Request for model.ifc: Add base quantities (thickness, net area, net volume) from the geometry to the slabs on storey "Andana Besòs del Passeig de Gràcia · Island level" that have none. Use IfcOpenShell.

First a look at what the model holds.

```python
import ifcopenshell
import ifcopenshell.util.element
import ifcopenshell.util.unit

model = ifcopenshell.open("model.ifc")
print(model.schema)
for unit_type in ("LENGTHUNIT", "AREAUNIT", "VOLUMEUNIT"):
    print(unit_type, ifcopenshell.util.unit.calculate_unit_scale(model, unit_type))
storey = next(s for s in model.by_type("IfcBuildingStorey") if s.Name == "Andana Besòs del Passeig de Gràcia · Island level")
slabs = [e for e in ifcopenshell.util.element.get_decomposition(storey) if e.is_a("IfcSlab")]
for e in sorted(slabs, key=lambda e: e.id()):
    print(e.id(), e.is_a(), e.Name, list(ifcopenshell.util.element.get_psets(e, qtos_only=True)), sep=" | ")
```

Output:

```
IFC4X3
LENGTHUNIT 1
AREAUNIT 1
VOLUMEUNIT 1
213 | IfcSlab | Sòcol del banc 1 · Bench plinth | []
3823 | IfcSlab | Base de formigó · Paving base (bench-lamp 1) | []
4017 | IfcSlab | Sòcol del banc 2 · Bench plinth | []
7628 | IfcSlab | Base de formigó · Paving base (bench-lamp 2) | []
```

```python
import ifcopenshell
import ifcopenshell.api.pset
import ifcopenshell.geom
import ifcopenshell.util.element
import ifcopenshell.util.shape
import ifcopenshell.util.unit

model = ifcopenshell.open("model.ifc")
unit_scale = ifcopenshell.util.unit.calculate_unit_scale(model)
area_scale = ifcopenshell.util.unit.calculate_unit_scale(model, "AREAUNIT")
volume_scale = ifcopenshell.util.unit.calculate_unit_scale(model, "VOLUMEUNIT")
settings = ifcopenshell.geom.settings()

storey = next(s for s in model.by_type("IfcBuildingStorey") if s.Name == "Andana Besòs del Passeig de Gràcia · Island level")
slabs = [e for e in ifcopenshell.util.element.get_decomposition(storey) if e.is_a("IfcSlab")]

for e in sorted(slabs, key=lambda e: e.id()):
    if ifcopenshell.util.element.get_psets(e, qtos_only=True, should_inherit=False):
        continue
    # Geometry comes back in metres, in the element's own axes.
    shape = ifcopenshell.geom.create_shape(settings, e)
    values = {
        "Width": ifcopenshell.util.shape.get_z(shape.geometry) / unit_scale,
        "NetArea": ifcopenshell.util.shape.get_footprint_area(shape.geometry) / area_scale,
        "NetVolume": ifcopenshell.util.shape.get_volume(shape.geometry) / volume_scale,
    }
    qto = ifcopenshell.api.pset.add_qto(model, product=e, name="Qto_SlabBaseQuantities")
    ifcopenshell.api.pset.edit_qto(model, qto=qto, properties=values)
    print(e.id(), {k: round(v, 3) for k, v in values.items()})

model.write("model_edited.ifc")
```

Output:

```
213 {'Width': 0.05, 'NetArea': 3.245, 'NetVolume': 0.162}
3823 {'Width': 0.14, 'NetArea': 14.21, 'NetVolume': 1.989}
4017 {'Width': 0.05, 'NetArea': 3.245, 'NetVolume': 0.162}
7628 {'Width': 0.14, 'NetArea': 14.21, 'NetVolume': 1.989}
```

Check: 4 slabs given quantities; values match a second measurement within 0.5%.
